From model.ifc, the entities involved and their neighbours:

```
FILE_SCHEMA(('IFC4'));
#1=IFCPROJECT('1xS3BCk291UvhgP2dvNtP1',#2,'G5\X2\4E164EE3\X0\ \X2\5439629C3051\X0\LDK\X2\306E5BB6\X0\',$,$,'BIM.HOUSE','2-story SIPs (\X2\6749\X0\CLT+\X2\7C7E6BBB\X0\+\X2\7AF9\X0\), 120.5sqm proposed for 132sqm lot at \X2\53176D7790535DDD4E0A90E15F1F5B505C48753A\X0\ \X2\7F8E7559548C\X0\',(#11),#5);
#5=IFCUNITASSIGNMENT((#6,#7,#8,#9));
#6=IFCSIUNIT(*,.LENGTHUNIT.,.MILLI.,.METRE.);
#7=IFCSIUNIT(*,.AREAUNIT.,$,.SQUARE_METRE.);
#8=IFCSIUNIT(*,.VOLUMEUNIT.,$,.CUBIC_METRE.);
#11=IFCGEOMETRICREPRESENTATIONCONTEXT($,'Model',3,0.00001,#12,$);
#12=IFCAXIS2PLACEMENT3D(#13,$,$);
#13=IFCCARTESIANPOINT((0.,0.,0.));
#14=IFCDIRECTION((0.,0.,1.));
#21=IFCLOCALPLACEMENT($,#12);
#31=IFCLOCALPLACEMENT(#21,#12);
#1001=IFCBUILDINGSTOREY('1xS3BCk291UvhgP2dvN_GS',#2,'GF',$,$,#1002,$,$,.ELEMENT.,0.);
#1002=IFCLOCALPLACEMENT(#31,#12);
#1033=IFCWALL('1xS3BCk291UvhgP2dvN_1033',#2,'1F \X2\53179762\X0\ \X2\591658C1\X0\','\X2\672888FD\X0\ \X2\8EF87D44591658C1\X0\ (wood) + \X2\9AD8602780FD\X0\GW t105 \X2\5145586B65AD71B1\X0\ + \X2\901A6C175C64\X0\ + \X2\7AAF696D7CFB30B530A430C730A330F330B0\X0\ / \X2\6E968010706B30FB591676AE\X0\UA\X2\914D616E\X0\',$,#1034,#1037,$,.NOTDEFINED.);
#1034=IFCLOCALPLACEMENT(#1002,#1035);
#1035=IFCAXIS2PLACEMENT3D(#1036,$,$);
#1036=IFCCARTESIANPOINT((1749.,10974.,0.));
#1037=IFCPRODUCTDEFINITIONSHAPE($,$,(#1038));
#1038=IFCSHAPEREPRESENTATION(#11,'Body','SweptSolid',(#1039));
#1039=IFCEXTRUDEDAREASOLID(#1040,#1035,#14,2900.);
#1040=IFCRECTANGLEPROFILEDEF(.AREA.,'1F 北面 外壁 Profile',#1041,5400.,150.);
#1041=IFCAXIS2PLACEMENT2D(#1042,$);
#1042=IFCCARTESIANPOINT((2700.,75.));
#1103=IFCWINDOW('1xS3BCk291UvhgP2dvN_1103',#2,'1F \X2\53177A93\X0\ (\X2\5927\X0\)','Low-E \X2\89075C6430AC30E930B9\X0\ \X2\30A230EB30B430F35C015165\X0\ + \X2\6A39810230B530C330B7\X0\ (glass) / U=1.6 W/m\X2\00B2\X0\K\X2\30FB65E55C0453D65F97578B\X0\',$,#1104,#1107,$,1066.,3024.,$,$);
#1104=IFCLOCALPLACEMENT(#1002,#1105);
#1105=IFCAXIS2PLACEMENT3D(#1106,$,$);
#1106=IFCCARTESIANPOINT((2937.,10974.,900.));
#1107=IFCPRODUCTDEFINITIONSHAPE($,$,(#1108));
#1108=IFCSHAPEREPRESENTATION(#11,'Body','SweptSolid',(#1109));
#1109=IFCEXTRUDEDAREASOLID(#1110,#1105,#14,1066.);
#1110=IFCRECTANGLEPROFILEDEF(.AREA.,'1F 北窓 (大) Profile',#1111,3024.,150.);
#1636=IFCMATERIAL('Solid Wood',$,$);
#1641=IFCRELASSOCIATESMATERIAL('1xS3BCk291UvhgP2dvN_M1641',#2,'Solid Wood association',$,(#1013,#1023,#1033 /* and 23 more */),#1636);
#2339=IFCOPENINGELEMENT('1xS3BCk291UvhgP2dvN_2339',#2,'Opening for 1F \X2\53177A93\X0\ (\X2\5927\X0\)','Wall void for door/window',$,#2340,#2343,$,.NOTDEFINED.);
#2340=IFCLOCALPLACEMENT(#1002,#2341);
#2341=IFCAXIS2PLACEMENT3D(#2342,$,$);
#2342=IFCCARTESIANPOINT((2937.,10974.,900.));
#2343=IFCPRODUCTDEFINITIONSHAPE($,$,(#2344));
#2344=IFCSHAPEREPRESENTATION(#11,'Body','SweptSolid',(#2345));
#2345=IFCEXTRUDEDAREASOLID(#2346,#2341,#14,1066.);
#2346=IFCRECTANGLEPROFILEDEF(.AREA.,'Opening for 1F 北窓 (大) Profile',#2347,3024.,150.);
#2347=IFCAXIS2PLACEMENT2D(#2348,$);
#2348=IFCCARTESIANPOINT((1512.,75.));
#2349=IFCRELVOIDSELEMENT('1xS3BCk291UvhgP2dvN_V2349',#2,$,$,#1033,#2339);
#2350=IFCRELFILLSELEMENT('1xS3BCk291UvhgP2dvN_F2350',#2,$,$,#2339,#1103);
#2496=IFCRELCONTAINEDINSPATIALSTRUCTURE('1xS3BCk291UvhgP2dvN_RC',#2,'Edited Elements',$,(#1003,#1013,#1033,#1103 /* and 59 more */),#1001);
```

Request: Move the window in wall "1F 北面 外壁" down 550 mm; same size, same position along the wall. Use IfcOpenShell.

```python
import numpy as np
import ifcopenshell
import ifcopenshell.api.geometry
import ifcopenshell.util.placement
import ifcopenshell.util.unit

model = ifcopenshell.open("model.ifc")
unit_scale = ifcopenshell.util.unit.calculate_unit_scale(model)

window = model.by_guid("1xS3BCk291UvhgP2dvN_1103")
opening = window.FillsVoids[0].RelatingOpeningElement
dz = -0.55 / unit_scale

shift = np.array([0.0, 0.0, dz])
# The window is not placed relative to its opening, so move both.
for product in (opening, window):
    matrix = ifcopenshell.util.placement.get_local_placement(product.ObjectPlacement)
    matrix[:3, 3] += shift
    ifcopenshell.api.geometry.edit_object_placement(model, product=product, matrix=matrix, is_si=False)

print(f"moved by {dz * unit_scale:+.3f} m")

model.write("model_v2.ifc")
```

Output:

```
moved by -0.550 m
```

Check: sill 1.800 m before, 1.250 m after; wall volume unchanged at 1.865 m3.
